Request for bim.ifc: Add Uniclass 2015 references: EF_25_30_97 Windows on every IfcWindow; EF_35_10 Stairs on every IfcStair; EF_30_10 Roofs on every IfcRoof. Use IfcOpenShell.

First a look at what the model holds.

```python
import ifcopenshell

model = ifcopenshell.open("bim.ifc")
print(model.schema)
print("classifications:", [c.Name for c in model.by_type("IfcClassification")])
for ifc_class in ("IfcDoor", "IfcRoof", "IfcStair", "IfcWall", "IfcWindow"):
    print(ifc_class, len(model.by_type(ifc_class)))
```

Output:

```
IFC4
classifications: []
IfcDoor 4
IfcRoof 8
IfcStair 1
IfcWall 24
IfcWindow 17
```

```python
import ifcopenshell
import ifcopenshell.api.classification

model = ifcopenshell.open("bim.ifc")

system = ifcopenshell.api.classification.add_classification(model, classification="Uniclass 2015")

codes = {
    "IfcWindow": ("EF_25_30_97", "Windows"),
    "IfcStair": ("EF_35_10", "Stairs"),
    "IfcRoof": ("EF_30_10", "Roofs"),
}
for ifc_class, (code, name) in codes.items():
    products = model.by_type(ifc_class)
    ifcopenshell.api.classification.add_reference(
        model, products=products, classification=system, identification=code, name=name
    )
    print(code, len(products))

model.write("bim_edited.ifc")
```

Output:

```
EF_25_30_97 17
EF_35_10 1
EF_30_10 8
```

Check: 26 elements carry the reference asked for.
